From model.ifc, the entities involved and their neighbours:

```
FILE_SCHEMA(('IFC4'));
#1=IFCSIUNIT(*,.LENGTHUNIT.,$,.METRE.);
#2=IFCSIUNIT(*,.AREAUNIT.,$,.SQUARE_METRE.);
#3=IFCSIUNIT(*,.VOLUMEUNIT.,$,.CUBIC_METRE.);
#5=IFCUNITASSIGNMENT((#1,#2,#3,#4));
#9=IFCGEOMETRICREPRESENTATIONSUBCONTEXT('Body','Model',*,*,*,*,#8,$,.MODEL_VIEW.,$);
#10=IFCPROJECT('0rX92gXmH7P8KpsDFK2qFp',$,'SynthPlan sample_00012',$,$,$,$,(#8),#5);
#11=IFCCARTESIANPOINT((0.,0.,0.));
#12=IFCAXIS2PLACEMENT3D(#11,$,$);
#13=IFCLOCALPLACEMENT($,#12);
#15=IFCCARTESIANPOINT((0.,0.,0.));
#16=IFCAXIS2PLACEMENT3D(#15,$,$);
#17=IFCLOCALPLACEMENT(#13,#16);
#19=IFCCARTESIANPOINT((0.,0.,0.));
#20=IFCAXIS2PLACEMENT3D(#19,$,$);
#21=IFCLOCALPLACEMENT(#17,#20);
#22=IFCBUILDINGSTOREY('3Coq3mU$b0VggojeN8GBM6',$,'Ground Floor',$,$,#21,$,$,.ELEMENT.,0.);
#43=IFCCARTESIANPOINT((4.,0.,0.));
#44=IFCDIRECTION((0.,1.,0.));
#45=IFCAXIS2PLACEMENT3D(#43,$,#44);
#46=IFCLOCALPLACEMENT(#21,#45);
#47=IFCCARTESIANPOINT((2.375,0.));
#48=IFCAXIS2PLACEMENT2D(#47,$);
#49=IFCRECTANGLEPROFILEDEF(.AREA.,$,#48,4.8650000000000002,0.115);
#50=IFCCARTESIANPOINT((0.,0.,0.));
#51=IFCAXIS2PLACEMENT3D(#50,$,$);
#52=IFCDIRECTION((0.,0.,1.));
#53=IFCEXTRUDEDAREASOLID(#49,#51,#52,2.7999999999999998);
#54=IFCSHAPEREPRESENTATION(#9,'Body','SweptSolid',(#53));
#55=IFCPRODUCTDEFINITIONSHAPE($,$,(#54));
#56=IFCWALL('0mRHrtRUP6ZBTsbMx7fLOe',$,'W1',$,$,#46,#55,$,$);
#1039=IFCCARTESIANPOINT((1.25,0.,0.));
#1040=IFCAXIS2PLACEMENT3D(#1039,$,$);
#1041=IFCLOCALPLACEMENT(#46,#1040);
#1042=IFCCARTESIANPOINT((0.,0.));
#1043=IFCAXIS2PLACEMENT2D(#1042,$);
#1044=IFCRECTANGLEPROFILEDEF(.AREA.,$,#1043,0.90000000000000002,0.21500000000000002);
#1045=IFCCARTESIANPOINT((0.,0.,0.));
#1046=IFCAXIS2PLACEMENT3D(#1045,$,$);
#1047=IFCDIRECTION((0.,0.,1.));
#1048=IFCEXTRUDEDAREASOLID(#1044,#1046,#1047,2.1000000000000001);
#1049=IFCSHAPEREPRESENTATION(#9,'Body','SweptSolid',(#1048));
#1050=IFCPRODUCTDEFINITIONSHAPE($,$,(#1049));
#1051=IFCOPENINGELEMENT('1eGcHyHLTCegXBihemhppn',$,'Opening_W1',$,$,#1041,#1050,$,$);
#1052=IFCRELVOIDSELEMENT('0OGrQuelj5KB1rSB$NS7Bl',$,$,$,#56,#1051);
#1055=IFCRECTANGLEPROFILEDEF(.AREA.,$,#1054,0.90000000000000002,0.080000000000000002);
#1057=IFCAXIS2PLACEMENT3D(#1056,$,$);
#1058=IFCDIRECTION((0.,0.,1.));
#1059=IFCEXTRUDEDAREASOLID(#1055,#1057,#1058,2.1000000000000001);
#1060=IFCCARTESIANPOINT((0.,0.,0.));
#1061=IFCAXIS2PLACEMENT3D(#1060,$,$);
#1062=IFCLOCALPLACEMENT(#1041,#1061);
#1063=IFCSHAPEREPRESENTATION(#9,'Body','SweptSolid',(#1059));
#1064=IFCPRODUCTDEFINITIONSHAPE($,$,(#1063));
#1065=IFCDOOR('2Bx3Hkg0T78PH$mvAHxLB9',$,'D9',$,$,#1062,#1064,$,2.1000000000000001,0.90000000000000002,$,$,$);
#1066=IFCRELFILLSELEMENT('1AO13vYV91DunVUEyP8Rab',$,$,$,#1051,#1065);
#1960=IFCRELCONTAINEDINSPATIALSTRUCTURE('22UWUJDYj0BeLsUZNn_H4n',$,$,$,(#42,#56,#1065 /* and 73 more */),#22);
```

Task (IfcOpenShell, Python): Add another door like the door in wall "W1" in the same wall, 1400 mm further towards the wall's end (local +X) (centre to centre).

```python
import ifcopenshell
import ifcopenshell.api.feature
import ifcopenshell.api.geometry
import ifcopenshell.api.root
import ifcopenshell.geom
import ifcopenshell.util.element
import ifcopenshell.util.placement
import ifcopenshell.util.shape
import ifcopenshell.util.unit

model = ifcopenshell.open("model.ifc")
unit_scale = ifcopenshell.util.unit.calculate_unit_scale(model)
settings = ifcopenshell.geom.settings()


def volume(element):
    """Net volume in cubic metres, openings subtracted."""
    shape = ifcopenshell.geom.create_shape(settings, element)
    return ifcopenshell.util.shape.get_volume(shape.geometry)


door = model.by_guid("2Bx3Hkg0T78PH$mvAHxLB9")
opening = door.FillsVoids[0].RelatingOpeningElement
wall = opening.VoidsElements[0].RelatingBuildingElement
before = volume(wall)
shift = ifcopenshell.util.placement.get_local_placement(wall.ObjectPlacement)[:3, 0] * 1.4 / unit_scale

# copy_class copies the void relationship, type, container and properties, but no geometry.
new_opening = ifcopenshell.api.root.copy_class(model, product=opening)
new_opening.Representation = ifcopenshell.util.element.copy_deep(
    model, opening.Representation, exclude=["IfcGeometricRepresentationContext", "IfcRepresentationMap"]
)
new_door = ifcopenshell.api.root.copy_class(model, product=door)
new_door.Representation = ifcopenshell.util.element.copy_deep(
    model, door.Representation, exclude=["IfcGeometricRepresentationContext", "IfcRepresentationMap"]
)
ifcopenshell.api.feature.add_filling(model, opening=new_opening, element=new_door)

for old, new in ((opening, new_opening), (door, new_door)):
    matrix = ifcopenshell.util.placement.get_local_placement(old.ObjectPlacement)
    matrix[:3, 3] += shift
    ifcopenshell.api.geometry.edit_object_placement(model, product=new, matrix=matrix, is_si=False)

after = volume(wall)

print(f"wall volume {before:.3f} -> {after:.3f} m3")

model.write("model-out.ifc")
```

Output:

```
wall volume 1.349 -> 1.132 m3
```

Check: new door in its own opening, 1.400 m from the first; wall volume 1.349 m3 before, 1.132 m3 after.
